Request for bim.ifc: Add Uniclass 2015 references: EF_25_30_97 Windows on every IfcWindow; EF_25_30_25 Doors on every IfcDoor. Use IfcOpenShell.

First a look at what the model holds.

```python
import ifcopenshell

model = ifcopenshell.open("bim.ifc")
print(model.schema)
print("classifications:", [c.Name for c in model.by_type("IfcClassification")])
for ifc_class in ("IfcDoor", "IfcRoof", "IfcStair", "IfcWall", "IfcWindow"):
    print(ifc_class, len(model.by_type(ifc_class)))
```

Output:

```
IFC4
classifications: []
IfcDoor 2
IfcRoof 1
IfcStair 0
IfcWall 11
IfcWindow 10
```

```python
import ifcopenshell
import ifcopenshell.api.classification

model = ifcopenshell.open("bim.ifc")

system = ifcopenshell.api.classification.add_classification(model, classification="Uniclass 2015")

codes = {
    "IfcWindow": ("EF_25_30_97", "Windows"),
    "IfcDoor": ("EF_25_30_25", "Doors"),
}
for ifc_class, (code, name) in codes.items():
    products = model.by_type(ifc_class)
    ifcopenshell.api.classification.add_reference(
        model, products=products, classification=system, identification=code, name=name
    )
    print(code, len(products))

model.write("bim_rev.ifc")
```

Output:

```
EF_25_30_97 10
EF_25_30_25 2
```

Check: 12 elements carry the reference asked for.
